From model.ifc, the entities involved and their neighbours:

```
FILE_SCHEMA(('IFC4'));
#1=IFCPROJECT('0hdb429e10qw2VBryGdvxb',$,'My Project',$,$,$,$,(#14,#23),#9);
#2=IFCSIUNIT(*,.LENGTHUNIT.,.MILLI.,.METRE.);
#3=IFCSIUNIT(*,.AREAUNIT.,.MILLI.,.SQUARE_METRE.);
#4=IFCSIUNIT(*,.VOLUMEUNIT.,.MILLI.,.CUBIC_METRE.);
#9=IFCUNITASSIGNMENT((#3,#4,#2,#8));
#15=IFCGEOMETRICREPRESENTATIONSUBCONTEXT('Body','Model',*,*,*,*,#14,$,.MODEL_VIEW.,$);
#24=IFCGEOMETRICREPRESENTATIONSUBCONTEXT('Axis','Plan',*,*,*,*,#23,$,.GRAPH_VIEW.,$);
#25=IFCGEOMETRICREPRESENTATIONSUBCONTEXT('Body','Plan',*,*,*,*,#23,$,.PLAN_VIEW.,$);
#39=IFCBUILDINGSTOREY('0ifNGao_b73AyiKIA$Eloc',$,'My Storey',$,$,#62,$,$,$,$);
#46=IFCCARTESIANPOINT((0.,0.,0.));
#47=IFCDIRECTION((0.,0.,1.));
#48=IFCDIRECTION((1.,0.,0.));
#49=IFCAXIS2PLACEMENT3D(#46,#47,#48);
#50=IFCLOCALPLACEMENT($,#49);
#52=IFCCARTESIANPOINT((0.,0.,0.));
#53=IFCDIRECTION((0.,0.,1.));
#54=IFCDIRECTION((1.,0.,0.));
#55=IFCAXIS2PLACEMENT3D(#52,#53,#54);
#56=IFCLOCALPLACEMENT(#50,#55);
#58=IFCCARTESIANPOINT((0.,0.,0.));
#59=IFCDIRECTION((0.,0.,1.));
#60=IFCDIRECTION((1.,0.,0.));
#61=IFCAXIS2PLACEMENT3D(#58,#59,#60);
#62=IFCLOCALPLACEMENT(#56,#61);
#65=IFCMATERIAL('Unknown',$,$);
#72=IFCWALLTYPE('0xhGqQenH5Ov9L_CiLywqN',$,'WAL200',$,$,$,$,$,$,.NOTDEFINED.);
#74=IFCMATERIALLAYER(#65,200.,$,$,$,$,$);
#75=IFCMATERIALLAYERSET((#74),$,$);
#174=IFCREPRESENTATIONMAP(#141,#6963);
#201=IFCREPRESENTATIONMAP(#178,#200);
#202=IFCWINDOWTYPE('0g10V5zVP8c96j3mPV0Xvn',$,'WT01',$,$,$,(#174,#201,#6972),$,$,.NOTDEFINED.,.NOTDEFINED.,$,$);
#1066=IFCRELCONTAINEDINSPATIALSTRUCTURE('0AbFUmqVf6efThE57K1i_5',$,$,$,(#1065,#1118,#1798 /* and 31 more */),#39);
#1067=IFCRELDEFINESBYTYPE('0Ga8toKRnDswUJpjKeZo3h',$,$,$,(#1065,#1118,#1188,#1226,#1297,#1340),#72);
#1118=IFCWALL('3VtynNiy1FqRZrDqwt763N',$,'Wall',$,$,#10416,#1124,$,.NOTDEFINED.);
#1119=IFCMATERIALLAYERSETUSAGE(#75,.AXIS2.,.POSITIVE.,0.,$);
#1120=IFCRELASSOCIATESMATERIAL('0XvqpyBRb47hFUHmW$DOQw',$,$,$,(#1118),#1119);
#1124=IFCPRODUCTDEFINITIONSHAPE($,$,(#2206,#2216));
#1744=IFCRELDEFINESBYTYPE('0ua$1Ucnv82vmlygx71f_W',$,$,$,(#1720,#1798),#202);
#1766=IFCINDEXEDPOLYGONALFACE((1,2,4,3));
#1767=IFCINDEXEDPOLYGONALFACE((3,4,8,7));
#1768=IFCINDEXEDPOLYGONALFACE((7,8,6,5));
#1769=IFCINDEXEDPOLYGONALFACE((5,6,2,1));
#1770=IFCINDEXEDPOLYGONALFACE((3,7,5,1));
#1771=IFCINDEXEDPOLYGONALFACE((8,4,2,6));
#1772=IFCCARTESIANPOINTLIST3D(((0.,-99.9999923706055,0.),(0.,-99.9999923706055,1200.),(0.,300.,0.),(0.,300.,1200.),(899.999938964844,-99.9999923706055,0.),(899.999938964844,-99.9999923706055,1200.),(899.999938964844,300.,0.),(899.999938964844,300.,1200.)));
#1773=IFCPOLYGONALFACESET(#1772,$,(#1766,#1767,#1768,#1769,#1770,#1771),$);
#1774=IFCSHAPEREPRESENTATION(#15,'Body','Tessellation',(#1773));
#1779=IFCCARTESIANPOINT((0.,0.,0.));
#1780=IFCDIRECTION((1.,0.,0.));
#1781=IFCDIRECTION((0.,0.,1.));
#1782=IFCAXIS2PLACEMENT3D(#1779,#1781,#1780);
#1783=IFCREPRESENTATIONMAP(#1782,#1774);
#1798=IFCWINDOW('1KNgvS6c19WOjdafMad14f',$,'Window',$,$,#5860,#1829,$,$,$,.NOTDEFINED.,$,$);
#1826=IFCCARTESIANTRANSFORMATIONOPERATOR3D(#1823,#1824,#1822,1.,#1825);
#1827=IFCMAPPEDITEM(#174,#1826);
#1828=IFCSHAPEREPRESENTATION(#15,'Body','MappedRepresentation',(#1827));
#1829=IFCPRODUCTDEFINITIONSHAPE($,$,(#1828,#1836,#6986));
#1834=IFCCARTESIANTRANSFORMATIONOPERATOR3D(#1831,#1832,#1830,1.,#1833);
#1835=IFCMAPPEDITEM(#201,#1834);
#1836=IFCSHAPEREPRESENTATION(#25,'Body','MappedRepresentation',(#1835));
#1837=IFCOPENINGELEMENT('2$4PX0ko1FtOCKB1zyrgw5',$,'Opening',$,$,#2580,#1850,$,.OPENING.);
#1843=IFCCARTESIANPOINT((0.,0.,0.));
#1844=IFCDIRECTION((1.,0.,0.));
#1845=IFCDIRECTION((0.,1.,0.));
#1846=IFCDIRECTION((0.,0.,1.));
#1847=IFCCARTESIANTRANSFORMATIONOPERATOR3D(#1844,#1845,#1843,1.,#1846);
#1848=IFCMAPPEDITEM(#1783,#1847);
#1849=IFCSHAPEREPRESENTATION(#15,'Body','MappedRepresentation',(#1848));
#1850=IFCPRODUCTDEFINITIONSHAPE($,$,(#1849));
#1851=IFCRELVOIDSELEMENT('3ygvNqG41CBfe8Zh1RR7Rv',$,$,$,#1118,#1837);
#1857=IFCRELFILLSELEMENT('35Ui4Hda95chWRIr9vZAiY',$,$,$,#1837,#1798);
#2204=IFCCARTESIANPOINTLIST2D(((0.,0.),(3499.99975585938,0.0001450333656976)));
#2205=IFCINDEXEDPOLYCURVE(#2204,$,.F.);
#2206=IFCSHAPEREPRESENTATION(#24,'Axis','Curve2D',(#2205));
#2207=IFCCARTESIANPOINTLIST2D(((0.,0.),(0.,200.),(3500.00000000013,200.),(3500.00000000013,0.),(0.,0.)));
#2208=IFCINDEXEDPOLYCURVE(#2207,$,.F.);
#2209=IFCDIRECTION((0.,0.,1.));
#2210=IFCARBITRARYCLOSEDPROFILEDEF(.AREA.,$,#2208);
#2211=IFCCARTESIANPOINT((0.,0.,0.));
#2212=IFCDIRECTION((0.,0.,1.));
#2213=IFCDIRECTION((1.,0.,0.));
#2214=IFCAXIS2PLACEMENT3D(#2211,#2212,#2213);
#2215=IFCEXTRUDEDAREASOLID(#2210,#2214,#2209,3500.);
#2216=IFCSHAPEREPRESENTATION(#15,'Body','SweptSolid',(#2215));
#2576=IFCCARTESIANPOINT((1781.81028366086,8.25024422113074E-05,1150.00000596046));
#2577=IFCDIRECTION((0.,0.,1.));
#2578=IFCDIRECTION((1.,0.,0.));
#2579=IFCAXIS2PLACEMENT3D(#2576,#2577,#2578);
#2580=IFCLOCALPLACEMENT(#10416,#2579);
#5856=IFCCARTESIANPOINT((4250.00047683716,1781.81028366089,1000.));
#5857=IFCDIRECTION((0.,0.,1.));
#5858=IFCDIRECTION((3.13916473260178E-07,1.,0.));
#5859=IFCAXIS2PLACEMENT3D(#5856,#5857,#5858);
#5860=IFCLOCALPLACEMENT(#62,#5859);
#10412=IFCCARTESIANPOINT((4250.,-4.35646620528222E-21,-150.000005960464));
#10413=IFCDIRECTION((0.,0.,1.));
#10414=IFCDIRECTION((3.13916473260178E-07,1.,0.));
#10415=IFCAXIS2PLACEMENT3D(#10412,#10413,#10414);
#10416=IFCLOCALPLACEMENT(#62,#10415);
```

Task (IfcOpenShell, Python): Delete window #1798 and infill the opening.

```python
import ifcopenshell
import ifcopenshell.api.feature
import ifcopenshell.api.root
import ifcopenshell.geom
import ifcopenshell.util.shape

model = ifcopenshell.open("model.ifc")
settings = ifcopenshell.geom.settings()


def volume(element):
    """Net volume in cubic metres, openings subtracted."""
    shape = ifcopenshell.geom.create_shape(settings, element)
    return ifcopenshell.util.shape.get_volume(shape.geometry)


window = model.by_guid("1KNgvS6c19WOjdafMad14f")
opening = window.FillsVoids[0].RelatingOpeningElement
wall = opening.VoidsElements[0].RelatingBuildingElement
before = volume(wall)

ifcopenshell.api.root.remove_product(model, product=window)
ifcopenshell.api.feature.remove_feature(model, feature=opening)

after = volume(wall)

print(f"wall volume {before:.3f} -> {after:.3f} m3")

model.write("model-out.ifc")
```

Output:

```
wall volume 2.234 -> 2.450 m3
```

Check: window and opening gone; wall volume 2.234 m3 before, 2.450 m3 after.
